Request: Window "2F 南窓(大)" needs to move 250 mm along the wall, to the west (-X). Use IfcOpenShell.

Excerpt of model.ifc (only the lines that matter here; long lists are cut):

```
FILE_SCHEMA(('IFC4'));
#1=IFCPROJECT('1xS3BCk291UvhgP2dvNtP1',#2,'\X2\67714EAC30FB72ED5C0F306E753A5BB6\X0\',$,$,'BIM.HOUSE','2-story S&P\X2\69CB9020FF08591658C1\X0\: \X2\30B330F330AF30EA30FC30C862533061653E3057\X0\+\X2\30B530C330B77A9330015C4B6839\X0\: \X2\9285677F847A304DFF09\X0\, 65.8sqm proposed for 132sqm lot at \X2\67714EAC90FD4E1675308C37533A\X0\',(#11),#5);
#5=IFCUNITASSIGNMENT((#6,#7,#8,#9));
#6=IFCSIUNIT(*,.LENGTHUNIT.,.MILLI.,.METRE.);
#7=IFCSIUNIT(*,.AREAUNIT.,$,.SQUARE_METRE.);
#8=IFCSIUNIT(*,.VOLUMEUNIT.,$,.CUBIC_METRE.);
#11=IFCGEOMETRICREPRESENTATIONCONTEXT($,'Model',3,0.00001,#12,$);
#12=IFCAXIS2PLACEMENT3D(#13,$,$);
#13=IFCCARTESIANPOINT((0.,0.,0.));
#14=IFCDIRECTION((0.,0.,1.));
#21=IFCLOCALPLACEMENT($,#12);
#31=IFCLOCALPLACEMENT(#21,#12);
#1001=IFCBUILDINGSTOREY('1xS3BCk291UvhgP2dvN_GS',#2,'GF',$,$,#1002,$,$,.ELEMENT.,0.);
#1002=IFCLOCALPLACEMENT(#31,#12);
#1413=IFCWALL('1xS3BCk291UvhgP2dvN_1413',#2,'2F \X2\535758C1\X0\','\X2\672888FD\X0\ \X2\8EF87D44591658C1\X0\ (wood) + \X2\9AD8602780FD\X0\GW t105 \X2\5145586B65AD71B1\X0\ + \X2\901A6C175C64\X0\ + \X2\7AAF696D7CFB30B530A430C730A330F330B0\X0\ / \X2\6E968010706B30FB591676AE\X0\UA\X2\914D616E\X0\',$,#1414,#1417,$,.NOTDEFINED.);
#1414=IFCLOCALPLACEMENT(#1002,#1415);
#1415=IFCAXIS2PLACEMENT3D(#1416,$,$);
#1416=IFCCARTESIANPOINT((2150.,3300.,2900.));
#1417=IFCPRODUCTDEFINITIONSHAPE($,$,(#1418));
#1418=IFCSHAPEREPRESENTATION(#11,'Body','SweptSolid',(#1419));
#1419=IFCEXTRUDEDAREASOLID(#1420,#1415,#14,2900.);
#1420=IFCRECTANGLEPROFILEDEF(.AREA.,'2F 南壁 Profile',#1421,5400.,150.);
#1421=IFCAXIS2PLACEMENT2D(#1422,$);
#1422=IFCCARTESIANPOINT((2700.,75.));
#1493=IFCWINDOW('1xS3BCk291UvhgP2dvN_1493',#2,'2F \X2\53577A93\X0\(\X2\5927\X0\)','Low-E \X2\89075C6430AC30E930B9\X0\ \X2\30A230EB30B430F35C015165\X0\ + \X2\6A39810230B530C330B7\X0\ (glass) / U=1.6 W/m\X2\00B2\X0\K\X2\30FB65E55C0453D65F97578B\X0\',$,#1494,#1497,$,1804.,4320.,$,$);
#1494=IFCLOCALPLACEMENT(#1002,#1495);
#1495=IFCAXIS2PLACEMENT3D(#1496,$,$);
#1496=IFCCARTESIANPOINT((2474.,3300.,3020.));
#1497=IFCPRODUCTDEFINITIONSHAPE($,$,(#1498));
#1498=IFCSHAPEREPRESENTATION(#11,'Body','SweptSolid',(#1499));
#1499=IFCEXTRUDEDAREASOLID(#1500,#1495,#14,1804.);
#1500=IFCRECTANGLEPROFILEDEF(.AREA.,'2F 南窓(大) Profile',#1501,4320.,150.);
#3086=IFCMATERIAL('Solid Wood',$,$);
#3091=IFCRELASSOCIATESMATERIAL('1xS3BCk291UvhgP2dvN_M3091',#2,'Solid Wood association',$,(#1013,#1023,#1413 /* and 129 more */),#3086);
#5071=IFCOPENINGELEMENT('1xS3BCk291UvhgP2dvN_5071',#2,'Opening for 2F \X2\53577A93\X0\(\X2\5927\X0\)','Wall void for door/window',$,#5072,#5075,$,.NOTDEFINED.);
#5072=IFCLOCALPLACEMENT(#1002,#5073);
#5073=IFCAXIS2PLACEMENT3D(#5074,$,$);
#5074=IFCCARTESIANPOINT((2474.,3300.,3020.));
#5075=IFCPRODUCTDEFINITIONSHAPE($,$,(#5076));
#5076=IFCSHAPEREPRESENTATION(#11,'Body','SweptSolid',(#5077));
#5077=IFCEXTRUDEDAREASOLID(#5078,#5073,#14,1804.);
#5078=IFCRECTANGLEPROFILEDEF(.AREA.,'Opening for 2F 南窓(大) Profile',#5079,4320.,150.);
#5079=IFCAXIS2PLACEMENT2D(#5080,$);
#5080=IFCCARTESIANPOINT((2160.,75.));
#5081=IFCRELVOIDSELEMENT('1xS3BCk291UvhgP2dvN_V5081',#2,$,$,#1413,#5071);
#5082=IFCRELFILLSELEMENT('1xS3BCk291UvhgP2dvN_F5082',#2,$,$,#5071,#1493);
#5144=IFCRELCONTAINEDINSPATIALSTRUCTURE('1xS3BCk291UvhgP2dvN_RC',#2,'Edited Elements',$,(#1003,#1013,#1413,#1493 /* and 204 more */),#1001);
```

```python
import ifcopenshell
import ifcopenshell.api.geometry
import ifcopenshell.util.placement

model = ifcopenshell.open("model.ifc")

window = model.by_id(1493)
opening = window.FillsVoids[0].RelatingOpeningElement
wall = opening.VoidsElements[0].RelatingBuildingElement

wall_matrix = ifcopenshell.util.placement.get_local_placement(wall.ObjectPlacement)
shift = wall_matrix[:3, 0] * -250.0
before = ifcopenshell.util.placement.get_local_placement(window.ObjectPlacement)[:3, 3].copy()

# The window is not placed relative to its opening, so move both.
for product in (opening, window):
    matrix = ifcopenshell.util.placement.get_local_placement(product.ObjectPlacement)
    matrix[:3, 3] += shift
    ifcopenshell.api.geometry.edit_object_placement(model, product=product, matrix=matrix, is_si=False)

after = ifcopenshell.util.placement.get_local_placement(window.ObjectPlacement)[:3, 3]
print("window moved by", (after - before).round(3) + 0.0)

model.write("model_edited.ifc")
```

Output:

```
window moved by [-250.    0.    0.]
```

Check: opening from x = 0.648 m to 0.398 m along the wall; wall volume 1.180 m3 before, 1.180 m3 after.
